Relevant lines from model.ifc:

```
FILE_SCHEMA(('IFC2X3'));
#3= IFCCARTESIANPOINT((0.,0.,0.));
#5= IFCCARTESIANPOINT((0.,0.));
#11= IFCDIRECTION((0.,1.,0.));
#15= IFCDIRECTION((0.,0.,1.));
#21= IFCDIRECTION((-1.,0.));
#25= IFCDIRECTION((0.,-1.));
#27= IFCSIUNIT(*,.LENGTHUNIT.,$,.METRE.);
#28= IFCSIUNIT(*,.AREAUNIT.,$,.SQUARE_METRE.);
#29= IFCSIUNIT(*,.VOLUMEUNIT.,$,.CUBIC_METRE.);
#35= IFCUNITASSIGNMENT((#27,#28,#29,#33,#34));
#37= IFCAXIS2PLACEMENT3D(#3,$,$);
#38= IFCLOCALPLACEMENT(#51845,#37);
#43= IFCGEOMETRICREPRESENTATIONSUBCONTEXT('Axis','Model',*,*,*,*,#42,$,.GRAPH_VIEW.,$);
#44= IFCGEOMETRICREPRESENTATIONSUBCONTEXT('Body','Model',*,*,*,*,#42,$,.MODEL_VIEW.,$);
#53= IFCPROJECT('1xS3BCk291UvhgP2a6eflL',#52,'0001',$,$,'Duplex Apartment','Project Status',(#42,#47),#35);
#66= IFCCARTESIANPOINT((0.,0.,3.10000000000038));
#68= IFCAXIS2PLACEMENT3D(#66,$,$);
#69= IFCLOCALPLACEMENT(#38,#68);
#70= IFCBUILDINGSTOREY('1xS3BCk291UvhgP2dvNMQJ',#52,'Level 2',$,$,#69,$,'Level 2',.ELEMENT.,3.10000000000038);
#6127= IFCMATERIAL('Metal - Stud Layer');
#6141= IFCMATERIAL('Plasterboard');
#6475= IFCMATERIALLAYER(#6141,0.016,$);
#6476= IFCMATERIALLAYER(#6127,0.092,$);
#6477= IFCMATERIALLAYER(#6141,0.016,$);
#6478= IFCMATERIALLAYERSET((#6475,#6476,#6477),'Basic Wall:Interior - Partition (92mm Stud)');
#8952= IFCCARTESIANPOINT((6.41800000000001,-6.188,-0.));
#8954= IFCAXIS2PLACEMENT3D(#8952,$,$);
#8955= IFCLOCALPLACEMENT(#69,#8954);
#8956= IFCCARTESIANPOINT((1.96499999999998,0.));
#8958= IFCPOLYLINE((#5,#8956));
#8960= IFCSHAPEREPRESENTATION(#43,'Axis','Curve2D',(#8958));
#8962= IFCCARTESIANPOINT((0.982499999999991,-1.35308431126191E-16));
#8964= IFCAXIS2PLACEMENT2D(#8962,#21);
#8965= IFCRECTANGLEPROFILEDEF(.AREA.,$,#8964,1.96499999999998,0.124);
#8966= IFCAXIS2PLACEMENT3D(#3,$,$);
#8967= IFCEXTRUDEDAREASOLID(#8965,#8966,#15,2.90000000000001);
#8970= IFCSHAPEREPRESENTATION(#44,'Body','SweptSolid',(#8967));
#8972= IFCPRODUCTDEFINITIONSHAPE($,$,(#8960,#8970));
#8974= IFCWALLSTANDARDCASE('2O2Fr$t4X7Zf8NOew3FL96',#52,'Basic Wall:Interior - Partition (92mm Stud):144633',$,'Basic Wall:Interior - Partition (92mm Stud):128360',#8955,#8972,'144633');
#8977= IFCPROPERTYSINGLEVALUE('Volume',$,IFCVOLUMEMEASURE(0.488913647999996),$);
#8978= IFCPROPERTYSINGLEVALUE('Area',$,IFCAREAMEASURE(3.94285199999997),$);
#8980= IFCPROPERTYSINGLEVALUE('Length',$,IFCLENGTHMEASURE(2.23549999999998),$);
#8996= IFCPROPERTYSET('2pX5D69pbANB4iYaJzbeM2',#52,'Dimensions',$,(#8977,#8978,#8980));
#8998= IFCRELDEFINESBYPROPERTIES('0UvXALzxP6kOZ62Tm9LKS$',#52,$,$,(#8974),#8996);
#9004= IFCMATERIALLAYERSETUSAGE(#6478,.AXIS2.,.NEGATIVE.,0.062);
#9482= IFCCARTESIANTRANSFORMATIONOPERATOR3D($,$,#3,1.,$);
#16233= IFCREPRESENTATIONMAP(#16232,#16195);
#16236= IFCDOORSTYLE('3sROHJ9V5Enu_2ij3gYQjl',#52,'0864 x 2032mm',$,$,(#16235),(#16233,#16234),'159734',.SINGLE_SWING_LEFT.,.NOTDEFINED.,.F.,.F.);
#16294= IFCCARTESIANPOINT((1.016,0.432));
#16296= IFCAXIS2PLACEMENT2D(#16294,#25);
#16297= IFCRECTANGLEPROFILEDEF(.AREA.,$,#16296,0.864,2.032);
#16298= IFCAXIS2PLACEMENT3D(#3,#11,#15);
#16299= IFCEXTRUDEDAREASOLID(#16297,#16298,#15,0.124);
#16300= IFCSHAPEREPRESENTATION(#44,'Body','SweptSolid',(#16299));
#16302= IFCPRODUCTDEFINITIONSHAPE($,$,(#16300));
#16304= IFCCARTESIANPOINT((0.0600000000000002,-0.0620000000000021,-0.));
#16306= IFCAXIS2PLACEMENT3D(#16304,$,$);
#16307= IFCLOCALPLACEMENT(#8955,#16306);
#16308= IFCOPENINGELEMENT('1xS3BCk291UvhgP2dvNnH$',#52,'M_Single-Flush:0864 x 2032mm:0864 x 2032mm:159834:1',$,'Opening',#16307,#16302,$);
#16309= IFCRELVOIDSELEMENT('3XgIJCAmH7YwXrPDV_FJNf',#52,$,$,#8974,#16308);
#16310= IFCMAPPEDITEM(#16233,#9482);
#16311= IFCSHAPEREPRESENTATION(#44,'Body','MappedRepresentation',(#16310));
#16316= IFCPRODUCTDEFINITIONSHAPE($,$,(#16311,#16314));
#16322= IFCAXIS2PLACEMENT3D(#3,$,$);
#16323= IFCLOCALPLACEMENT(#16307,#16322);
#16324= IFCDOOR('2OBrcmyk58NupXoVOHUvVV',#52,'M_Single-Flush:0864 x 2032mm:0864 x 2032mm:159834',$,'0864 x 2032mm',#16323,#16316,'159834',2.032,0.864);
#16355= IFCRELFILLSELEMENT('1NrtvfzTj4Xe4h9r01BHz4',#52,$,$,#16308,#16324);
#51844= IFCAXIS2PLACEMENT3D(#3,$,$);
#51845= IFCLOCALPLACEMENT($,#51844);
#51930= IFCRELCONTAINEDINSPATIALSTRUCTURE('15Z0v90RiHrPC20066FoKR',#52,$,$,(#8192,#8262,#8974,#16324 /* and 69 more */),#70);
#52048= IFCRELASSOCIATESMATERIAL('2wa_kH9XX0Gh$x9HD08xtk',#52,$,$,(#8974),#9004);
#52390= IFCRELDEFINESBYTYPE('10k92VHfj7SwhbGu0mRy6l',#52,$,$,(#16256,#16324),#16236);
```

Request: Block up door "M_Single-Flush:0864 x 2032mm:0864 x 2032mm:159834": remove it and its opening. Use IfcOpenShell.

```python
import ifcopenshell
import ifcopenshell.api.feature
import ifcopenshell.api.pset
import ifcopenshell.api.root
import ifcopenshell.geom
import ifcopenshell.util.element
import ifcopenshell.util.shape
import ifcopenshell.util.unit

model = ifcopenshell.open("model.ifc")
area_scale = ifcopenshell.util.unit.calculate_unit_scale(model, "AREAUNIT")
volume_scale = ifcopenshell.util.unit.calculate_unit_scale(model, "VOLUMEUNIT")
settings = ifcopenshell.geom.settings()


def volume(element):
    """Net volume in cubic metres, openings subtracted."""
    shape = ifcopenshell.geom.create_shape(settings, element)
    return ifcopenshell.util.shape.get_volume(shape.geometry)


door = model.by_id(16324)
opening = door.FillsVoids[0].RelatingOpeningElement
wall = opening.VoidsElements[0].RelatingBuildingElement
before = volume(wall)

ifcopenshell.api.root.remove_product(model, product=door)
ifcopenshell.api.feature.remove_feature(model, feature=opening)

after = volume(wall)
thickness = 0.124  # wall thickness in metres

# Update the wall's stored quantities.
pset = model.by_id(ifcopenshell.util.element.get_pset(wall, "Dimensions", should_inherit=False)["id"])
ifcopenshell.api.pset.edit_pset(model, pset=pset, properties={
    "Volume": model.create_entity("IfcVolumeMeasure", after / volume_scale),
    "Area": model.create_entity("IfcAreaMeasure", after / thickness / area_scale),
})

print(f"wall volume {before:.3f} -> {after:.3f} m3")

model.write("model-out.ifc")
```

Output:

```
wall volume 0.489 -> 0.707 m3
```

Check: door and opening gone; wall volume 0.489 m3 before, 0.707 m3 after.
